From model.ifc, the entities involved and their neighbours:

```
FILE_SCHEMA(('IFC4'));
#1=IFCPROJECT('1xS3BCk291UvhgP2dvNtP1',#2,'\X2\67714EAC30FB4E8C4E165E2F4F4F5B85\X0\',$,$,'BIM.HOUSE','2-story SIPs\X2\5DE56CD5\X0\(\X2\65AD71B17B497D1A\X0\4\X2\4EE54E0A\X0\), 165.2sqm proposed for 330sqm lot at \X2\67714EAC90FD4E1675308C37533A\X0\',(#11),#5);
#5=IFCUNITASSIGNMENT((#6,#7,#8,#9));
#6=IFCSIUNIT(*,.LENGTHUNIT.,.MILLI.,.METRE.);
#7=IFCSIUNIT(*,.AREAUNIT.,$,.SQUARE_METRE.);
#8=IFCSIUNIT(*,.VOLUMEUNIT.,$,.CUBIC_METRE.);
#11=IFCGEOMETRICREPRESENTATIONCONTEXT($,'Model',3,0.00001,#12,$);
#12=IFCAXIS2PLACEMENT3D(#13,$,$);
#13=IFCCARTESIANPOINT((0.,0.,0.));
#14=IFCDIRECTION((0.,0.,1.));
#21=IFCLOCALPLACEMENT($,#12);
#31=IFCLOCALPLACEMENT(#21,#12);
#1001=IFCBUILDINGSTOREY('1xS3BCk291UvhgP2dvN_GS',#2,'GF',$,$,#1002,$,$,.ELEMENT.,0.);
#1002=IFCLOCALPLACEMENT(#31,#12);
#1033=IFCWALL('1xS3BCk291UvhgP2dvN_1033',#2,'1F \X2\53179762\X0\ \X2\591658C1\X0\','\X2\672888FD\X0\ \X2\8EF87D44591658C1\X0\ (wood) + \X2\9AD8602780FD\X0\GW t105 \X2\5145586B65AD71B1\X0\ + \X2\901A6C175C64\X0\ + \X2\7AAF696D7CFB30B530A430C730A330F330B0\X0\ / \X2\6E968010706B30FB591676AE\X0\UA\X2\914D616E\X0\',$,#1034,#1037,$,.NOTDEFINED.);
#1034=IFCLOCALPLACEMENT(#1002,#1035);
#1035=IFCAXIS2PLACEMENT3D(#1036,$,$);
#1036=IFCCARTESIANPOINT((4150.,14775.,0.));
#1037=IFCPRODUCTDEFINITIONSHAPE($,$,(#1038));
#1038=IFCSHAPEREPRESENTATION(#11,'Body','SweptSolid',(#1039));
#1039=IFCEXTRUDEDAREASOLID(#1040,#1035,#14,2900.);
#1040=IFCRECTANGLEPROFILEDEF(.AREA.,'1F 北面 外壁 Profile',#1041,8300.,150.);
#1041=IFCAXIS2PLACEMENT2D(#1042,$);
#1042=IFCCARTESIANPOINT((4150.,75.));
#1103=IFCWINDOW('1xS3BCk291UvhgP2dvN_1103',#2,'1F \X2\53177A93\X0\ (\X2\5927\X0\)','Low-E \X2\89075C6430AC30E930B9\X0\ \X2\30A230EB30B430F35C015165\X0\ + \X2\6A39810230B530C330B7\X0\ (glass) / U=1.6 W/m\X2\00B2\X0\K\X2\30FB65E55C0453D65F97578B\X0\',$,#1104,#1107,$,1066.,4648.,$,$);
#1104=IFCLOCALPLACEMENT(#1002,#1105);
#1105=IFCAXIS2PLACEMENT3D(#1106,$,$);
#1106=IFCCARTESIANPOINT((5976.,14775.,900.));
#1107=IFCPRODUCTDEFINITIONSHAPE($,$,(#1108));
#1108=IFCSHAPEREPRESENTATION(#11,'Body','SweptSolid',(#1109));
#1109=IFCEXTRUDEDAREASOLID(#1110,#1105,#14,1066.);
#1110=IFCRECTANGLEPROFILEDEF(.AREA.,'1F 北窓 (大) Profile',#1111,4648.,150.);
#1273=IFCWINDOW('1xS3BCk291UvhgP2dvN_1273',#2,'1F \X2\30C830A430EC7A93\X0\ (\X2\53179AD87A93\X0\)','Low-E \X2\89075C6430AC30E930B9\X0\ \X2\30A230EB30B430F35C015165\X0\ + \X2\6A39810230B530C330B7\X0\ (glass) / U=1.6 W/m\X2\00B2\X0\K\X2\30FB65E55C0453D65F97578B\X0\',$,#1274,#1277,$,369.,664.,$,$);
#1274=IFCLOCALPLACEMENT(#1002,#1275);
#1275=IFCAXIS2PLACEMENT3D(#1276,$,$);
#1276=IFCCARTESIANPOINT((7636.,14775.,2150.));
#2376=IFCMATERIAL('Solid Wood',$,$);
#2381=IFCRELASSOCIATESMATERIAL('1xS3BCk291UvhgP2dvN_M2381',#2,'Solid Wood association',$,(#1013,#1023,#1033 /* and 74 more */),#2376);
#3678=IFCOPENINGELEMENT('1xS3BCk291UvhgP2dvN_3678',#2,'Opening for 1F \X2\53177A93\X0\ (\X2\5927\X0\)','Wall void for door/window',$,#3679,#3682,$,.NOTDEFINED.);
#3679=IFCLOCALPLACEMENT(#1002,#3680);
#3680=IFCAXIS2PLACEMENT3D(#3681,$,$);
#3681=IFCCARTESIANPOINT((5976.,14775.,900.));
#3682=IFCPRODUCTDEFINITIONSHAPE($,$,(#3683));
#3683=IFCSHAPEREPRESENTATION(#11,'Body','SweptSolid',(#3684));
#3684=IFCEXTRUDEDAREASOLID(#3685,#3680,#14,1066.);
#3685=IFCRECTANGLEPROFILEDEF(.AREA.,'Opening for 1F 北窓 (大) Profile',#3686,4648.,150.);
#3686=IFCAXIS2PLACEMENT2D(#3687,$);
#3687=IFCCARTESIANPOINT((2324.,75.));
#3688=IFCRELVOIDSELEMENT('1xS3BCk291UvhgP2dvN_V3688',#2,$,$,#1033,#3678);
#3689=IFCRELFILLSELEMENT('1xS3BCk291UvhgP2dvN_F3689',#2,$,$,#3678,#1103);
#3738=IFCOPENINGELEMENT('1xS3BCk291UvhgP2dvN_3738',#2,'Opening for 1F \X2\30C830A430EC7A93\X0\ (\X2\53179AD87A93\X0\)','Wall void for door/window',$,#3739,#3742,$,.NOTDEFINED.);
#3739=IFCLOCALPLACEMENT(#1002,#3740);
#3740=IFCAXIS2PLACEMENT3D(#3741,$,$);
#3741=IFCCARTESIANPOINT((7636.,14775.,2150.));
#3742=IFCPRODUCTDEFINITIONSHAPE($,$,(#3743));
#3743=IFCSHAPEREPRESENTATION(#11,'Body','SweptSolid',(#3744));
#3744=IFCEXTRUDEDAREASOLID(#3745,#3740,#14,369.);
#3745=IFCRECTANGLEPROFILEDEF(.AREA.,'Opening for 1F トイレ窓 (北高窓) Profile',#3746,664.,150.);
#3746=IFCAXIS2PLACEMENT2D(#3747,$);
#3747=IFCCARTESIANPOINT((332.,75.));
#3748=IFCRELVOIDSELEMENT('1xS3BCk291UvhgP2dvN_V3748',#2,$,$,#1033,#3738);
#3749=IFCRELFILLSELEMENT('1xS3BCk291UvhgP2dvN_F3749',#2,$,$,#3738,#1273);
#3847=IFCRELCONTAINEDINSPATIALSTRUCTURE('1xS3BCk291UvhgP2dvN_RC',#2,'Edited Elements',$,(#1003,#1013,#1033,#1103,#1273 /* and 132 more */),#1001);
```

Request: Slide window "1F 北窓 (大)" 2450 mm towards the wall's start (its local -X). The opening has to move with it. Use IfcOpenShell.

```python
import ifcopenshell
import ifcopenshell.api.geometry
import ifcopenshell.util.placement
import ifcopenshell.util.unit

model = ifcopenshell.open("model.ifc")
unit_scale = ifcopenshell.util.unit.calculate_unit_scale(model)

window = model.by_id(1103)
opening = window.FillsVoids[0].RelatingOpeningElement
wall = opening.VoidsElements[0].RelatingBuildingElement

wall_matrix = ifcopenshell.util.placement.get_local_placement(wall.ObjectPlacement)
shift = wall_matrix[:3, 0] * -2.45 / unit_scale
before = ifcopenshell.util.placement.get_local_placement(window.ObjectPlacement)[:3, 3].copy()

# The window is not placed relative to its opening, so move both.
for product in (opening, window):
    matrix = ifcopenshell.util.placement.get_local_placement(product.ObjectPlacement)
    matrix[:3, 3] += shift
    ifcopenshell.api.geometry.edit_object_placement(model, product=product, matrix=matrix, is_si=False)

after = ifcopenshell.util.placement.get_local_placement(window.ObjectPlacement)[:3, 3]
print("window moved by", (after - before).round(3) + 0.0)

model.write("model-out.ifc")
```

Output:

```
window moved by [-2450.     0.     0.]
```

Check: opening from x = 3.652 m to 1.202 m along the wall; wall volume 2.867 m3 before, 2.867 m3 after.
